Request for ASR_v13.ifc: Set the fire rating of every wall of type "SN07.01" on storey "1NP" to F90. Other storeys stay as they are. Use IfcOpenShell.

First a look at what the model holds.

```python
import ifcopenshell
import ifcopenshell.util.element

model = ifcopenshell.open("ASR_v13.ifc")
print(model.schema)
storey = next(s for s in model.by_type("IfcBuildingStorey") if s.Name == "1NP")
walls = [e for e in ifcopenshell.util.element.get_decomposition(storey) if e.is_a("IfcWall")]
seen = {}
for e in walls:
    element_type = ifcopenshell.util.element.get_type(e)
    key = (element_type.Name if element_type != e and element_type else None, ifcopenshell.util.element.get_pset(e, "Pset_WallCommon", "FireRating"))
    seen[key] = seen.get(key, 0) + 1
for (name, value), count in sorted(seen.items(), key=str):
    print(count, "x", name, "|", value)
```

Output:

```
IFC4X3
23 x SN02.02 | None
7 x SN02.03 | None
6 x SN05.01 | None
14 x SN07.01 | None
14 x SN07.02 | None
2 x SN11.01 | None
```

```python
import ifcopenshell
import ifcopenshell.api.pset
import ifcopenshell.util.element

model = ifcopenshell.open("ASR_v13.ifc")

storey = next(s for s in model.by_type("IfcBuildingStorey") if s.Name == "1NP")
walls = [e for e in ifcopenshell.util.element.get_decomposition(storey) if e.is_a("IfcWall")]

count = 0
for e in walls:
    element_type = ifcopenshell.util.element.get_type(e)
    if element_type in (None, e) or element_type.Name != "SN07.01":
        continue
    # add_pset returns the element's existing set when there is one.
    pset = ifcopenshell.api.pset.add_pset(model, product=e, name="Pset_WallCommon")
    ifcopenshell.api.pset.edit_pset(model, pset=pset, properties={"FireRating": "F90"})
    count += 1

print(count, "walls updated")

model.write("ASR_v13_edited.ifc")
```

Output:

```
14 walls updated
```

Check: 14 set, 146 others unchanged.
